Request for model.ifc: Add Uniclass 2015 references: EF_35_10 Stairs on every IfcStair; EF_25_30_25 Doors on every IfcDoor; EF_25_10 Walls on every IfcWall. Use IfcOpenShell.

First a look at what the model holds.

```python
import ifcopenshell

model = ifcopenshell.open("model.ifc")
print(model.schema)
print("classifications:", [c.Name for c in model.by_type("IfcClassification")])
for ifc_class in ("IfcDoor", "IfcRoof", "IfcStair", "IfcWall", "IfcWindow"):
    print(ifc_class, len(model.by_type(ifc_class)))
```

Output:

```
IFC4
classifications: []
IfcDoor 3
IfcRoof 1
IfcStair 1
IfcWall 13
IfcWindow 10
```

```python
import ifcopenshell
import ifcopenshell.api.classification

model = ifcopenshell.open("model.ifc")

system = ifcopenshell.api.classification.add_classification(model, classification="Uniclass 2015")

codes = {
    "IfcStair": ("EF_35_10", "Stairs"),
    "IfcDoor": ("EF_25_30_25", "Doors"),
    "IfcWall": ("EF_25_10", "Walls"),
}
for ifc_class, (code, name) in codes.items():
    products = model.by_type(ifc_class)
    ifcopenshell.api.classification.add_reference(
        model, products=products, classification=system, identification=code, name=name
    )
    print(code, len(products))

model.write("model_updated.ifc")
```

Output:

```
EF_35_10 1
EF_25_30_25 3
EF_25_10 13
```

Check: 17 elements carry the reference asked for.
